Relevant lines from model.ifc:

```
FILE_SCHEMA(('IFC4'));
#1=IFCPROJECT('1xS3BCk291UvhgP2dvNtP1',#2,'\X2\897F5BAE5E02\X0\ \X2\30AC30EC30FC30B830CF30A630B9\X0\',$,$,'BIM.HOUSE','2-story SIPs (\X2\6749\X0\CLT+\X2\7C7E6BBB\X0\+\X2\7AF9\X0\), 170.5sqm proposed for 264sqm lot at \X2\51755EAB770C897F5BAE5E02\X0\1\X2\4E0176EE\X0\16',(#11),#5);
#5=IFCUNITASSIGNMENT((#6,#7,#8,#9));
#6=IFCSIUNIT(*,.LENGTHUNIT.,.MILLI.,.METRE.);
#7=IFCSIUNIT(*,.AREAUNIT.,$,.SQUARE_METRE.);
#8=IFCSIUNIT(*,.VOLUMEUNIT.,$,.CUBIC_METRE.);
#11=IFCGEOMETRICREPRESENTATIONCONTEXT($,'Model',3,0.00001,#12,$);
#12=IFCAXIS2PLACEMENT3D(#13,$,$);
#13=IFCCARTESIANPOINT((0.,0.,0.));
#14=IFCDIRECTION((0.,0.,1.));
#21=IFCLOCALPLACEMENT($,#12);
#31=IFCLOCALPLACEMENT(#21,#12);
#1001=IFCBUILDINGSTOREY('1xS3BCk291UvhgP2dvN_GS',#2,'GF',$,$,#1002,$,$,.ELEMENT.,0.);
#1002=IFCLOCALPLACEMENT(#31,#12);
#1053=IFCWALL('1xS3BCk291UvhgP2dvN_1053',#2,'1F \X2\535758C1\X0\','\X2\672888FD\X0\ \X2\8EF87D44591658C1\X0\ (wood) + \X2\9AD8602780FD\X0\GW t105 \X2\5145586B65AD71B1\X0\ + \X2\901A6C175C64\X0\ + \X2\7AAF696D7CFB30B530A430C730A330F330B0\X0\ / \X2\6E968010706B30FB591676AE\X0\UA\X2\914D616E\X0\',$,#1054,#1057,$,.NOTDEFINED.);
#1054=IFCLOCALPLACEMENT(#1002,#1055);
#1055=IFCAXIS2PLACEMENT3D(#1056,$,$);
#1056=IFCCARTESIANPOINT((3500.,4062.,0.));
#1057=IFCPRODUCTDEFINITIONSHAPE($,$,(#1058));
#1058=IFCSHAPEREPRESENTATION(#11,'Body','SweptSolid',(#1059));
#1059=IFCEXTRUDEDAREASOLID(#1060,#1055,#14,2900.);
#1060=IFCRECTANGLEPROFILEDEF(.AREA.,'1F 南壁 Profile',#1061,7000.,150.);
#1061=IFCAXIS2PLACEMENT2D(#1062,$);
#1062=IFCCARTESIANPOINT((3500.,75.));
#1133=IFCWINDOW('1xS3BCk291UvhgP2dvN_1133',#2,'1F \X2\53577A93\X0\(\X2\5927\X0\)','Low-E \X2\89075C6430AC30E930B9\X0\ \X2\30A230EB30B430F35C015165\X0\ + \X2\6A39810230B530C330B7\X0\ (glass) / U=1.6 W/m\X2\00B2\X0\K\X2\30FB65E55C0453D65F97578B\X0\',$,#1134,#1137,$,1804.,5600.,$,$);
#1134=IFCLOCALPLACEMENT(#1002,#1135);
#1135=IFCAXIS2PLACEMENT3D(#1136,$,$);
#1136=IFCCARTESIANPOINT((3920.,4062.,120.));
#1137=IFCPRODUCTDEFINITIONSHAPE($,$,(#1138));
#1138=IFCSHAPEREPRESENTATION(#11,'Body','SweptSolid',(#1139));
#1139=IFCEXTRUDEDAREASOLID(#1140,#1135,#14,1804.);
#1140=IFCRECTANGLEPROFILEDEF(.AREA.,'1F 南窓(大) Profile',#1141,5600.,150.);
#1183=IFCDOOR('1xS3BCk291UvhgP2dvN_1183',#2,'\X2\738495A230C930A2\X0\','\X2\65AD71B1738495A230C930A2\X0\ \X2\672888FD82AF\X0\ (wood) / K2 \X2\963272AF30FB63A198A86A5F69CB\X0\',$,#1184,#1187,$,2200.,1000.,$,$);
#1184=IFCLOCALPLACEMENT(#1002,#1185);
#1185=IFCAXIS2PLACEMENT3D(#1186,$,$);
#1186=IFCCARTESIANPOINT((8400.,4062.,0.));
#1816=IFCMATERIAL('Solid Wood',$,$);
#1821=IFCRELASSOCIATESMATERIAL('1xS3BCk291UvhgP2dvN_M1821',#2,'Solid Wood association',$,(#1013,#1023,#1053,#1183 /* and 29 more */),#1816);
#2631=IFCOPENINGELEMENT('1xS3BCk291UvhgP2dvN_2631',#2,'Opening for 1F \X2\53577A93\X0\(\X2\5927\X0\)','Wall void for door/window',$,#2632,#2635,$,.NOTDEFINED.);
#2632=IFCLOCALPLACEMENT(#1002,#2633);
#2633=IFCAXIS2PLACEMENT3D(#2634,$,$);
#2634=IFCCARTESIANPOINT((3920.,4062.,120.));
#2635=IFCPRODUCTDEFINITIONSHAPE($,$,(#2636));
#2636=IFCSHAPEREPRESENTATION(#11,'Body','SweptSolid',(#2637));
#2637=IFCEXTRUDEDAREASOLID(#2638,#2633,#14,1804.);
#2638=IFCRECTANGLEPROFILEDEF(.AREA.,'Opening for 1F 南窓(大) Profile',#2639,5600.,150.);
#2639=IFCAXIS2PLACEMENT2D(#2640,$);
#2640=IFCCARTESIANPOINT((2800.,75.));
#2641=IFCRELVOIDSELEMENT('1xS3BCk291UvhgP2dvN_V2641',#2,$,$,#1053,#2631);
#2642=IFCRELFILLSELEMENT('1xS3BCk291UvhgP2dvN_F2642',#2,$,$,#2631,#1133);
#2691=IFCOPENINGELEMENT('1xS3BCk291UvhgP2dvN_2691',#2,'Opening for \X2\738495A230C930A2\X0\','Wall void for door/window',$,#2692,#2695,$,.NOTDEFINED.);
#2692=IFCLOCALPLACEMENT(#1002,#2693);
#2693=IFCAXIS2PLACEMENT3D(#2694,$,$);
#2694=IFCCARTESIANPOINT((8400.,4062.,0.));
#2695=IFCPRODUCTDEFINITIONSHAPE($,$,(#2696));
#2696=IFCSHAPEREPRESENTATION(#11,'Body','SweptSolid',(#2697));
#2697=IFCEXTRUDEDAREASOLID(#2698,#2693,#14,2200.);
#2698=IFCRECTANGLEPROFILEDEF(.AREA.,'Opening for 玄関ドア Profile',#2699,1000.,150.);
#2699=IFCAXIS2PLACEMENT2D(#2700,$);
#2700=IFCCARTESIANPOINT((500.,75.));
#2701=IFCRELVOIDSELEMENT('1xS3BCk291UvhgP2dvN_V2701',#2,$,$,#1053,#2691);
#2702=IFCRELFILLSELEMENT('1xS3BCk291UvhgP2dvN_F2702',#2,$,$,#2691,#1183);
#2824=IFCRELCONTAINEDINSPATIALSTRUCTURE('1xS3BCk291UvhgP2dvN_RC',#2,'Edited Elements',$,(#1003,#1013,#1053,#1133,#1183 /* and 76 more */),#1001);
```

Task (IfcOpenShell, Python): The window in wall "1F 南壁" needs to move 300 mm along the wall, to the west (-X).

```python
import ifcopenshell
import ifcopenshell.api.geometry
import ifcopenshell.util.placement

model = ifcopenshell.open("model.ifc")

window = model.by_id(1133)
opening = window.FillsVoids[0].RelatingOpeningElement
wall = opening.VoidsElements[0].RelatingBuildingElement

wall_matrix = ifcopenshell.util.placement.get_local_placement(wall.ObjectPlacement)
shift = wall_matrix[:3, 0] * -300.0
before = ifcopenshell.util.placement.get_local_placement(window.ObjectPlacement)[:3, 3].copy()

# The window is not placed relative to its opening, so move both.
for product in (opening, window):
    matrix = ifcopenshell.util.placement.get_local_placement(product.ObjectPlacement)
    matrix[:3, 3] += shift
    ifcopenshell.api.geometry.edit_object_placement(model, product=product, matrix=matrix, is_si=False)

after = ifcopenshell.util.placement.get_local_placement(window.ObjectPlacement)[:3, 3]
print("window moved by", (after - before).round(3) + 0.0)

model.write("model_updated.ifc")
```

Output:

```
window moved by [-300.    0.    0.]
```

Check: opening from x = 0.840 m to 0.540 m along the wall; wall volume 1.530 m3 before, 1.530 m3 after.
